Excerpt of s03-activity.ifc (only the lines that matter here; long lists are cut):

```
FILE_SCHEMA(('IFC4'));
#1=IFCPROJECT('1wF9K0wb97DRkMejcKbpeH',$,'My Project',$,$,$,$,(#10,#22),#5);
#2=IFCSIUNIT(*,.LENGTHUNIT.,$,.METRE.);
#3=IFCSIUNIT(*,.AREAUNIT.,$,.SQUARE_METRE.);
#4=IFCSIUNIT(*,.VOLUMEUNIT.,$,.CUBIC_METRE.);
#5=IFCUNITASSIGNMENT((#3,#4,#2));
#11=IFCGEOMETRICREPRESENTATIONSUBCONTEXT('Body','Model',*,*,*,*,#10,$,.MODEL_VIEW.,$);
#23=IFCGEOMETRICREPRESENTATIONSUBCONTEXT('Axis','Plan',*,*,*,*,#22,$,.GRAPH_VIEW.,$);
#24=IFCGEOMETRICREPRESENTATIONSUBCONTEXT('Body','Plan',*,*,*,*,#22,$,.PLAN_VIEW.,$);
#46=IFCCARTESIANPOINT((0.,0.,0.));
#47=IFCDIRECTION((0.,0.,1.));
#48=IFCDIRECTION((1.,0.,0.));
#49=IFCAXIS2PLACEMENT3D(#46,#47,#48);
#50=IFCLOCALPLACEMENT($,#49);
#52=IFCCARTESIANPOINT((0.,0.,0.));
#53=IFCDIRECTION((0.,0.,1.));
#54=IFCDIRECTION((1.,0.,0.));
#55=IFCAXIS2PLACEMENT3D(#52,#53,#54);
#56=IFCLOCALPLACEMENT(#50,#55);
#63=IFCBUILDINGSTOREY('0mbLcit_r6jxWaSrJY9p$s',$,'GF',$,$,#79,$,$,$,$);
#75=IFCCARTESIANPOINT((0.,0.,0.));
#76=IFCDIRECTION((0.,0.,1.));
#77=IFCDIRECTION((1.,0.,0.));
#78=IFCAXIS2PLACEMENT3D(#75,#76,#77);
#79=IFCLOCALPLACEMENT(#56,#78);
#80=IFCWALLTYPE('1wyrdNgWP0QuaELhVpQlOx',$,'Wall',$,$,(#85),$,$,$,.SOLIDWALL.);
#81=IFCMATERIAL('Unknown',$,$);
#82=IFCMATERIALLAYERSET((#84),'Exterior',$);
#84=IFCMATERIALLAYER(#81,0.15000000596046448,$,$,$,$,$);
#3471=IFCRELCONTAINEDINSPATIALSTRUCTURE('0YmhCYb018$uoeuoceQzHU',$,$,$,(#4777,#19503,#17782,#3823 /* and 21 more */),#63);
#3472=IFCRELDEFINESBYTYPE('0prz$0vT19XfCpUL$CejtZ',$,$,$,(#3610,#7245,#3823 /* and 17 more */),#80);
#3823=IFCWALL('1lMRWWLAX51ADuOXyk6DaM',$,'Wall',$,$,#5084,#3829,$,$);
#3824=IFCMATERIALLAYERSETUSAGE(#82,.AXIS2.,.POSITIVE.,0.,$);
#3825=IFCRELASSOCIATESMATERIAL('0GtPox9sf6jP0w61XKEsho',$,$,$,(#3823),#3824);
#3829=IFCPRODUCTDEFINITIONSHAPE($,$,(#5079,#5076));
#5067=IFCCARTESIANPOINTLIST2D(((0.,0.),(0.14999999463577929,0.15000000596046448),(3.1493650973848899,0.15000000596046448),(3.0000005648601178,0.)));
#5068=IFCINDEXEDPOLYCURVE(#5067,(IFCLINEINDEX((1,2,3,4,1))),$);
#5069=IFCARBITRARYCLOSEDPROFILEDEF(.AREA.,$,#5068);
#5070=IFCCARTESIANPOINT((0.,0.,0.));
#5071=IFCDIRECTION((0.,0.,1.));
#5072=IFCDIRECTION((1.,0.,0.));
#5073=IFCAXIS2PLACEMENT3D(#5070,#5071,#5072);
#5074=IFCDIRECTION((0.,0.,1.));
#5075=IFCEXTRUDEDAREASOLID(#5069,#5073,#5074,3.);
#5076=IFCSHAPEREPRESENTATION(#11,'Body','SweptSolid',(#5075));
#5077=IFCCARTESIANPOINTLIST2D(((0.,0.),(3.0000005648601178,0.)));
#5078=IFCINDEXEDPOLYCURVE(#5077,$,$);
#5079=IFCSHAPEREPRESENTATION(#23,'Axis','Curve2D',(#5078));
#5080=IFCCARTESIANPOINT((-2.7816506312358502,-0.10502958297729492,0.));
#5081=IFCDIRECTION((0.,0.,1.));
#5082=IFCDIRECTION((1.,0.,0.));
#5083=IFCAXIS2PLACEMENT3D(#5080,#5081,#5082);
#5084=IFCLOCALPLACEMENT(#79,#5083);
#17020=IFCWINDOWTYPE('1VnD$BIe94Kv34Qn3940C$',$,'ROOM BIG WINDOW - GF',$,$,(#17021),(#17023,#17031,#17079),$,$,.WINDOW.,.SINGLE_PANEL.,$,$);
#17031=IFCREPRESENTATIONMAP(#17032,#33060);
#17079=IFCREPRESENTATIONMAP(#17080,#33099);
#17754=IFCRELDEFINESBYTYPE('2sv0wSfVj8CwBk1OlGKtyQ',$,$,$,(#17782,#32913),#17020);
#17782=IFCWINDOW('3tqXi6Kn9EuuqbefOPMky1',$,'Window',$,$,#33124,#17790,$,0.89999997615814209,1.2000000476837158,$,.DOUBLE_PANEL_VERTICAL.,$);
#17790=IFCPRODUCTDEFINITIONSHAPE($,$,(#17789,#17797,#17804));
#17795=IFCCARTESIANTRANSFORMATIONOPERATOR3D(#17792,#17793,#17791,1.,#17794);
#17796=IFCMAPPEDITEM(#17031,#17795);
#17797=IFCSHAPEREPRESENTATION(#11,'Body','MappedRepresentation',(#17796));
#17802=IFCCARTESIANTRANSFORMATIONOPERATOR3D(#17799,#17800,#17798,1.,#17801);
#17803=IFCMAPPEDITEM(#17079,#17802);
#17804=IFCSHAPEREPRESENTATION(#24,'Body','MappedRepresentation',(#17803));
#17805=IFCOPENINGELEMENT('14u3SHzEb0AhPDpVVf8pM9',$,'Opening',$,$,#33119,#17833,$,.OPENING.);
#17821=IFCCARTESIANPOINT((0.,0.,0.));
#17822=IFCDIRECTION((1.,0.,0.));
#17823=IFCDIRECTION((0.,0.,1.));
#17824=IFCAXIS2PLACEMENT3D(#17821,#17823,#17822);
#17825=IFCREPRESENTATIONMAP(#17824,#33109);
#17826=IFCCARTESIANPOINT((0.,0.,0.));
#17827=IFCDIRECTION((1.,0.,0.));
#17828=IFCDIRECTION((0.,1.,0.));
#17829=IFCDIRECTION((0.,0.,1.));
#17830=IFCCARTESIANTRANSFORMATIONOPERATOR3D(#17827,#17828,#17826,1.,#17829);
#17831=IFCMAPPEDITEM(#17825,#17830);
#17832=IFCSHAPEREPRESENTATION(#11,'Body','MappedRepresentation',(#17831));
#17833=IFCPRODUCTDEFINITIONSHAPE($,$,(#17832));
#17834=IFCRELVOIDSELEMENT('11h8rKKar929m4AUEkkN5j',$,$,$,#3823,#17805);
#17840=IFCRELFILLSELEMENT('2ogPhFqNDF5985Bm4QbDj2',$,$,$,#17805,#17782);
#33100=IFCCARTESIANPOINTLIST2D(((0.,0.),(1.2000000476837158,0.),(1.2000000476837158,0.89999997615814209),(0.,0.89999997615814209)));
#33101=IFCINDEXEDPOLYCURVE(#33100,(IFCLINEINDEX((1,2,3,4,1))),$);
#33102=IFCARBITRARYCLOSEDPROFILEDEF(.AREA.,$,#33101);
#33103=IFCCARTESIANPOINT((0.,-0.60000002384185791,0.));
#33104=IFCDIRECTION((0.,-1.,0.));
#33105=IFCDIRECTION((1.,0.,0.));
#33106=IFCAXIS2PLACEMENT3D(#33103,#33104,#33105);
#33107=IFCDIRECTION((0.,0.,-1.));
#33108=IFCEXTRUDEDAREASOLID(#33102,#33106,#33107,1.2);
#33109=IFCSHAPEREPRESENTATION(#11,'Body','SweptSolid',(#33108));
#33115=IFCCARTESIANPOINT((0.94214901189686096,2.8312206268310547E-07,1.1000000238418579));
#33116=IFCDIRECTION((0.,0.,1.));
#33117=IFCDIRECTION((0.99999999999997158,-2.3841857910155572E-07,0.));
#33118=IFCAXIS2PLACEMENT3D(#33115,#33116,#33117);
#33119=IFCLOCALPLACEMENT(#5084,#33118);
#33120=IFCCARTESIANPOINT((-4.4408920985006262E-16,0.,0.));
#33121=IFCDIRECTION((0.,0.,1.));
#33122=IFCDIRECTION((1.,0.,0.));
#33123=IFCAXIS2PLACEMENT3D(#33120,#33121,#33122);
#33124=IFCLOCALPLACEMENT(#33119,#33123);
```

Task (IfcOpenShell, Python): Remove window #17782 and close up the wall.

```python
import ifcopenshell
import ifcopenshell.api.feature
import ifcopenshell.api.root
import ifcopenshell.geom
import ifcopenshell.util.shape

model = ifcopenshell.open("s03-activity.ifc")
settings = ifcopenshell.geom.settings()


def volume(element):
    """Net volume in cubic metres, openings subtracted."""
    shape = ifcopenshell.geom.create_shape(settings, element)
    return ifcopenshell.util.shape.get_volume(shape.geometry)


window = model.by_guid("3tqXi6Kn9EuuqbefOPMky1")
opening = window.FillsVoids[0].RelatingOpeningElement
wall = opening.VoidsElements[0].RelatingBuildingElement
before = volume(wall)

ifcopenshell.api.root.remove_product(model, product=window)
ifcopenshell.api.feature.remove_feature(model, feature=opening)

after = volume(wall)

print(f"wall volume {before:.3f} -> {after:.3f} m3")

model.write("s03-activity_updated.ifc")
```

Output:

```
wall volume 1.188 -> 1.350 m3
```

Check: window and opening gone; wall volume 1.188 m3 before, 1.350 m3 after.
